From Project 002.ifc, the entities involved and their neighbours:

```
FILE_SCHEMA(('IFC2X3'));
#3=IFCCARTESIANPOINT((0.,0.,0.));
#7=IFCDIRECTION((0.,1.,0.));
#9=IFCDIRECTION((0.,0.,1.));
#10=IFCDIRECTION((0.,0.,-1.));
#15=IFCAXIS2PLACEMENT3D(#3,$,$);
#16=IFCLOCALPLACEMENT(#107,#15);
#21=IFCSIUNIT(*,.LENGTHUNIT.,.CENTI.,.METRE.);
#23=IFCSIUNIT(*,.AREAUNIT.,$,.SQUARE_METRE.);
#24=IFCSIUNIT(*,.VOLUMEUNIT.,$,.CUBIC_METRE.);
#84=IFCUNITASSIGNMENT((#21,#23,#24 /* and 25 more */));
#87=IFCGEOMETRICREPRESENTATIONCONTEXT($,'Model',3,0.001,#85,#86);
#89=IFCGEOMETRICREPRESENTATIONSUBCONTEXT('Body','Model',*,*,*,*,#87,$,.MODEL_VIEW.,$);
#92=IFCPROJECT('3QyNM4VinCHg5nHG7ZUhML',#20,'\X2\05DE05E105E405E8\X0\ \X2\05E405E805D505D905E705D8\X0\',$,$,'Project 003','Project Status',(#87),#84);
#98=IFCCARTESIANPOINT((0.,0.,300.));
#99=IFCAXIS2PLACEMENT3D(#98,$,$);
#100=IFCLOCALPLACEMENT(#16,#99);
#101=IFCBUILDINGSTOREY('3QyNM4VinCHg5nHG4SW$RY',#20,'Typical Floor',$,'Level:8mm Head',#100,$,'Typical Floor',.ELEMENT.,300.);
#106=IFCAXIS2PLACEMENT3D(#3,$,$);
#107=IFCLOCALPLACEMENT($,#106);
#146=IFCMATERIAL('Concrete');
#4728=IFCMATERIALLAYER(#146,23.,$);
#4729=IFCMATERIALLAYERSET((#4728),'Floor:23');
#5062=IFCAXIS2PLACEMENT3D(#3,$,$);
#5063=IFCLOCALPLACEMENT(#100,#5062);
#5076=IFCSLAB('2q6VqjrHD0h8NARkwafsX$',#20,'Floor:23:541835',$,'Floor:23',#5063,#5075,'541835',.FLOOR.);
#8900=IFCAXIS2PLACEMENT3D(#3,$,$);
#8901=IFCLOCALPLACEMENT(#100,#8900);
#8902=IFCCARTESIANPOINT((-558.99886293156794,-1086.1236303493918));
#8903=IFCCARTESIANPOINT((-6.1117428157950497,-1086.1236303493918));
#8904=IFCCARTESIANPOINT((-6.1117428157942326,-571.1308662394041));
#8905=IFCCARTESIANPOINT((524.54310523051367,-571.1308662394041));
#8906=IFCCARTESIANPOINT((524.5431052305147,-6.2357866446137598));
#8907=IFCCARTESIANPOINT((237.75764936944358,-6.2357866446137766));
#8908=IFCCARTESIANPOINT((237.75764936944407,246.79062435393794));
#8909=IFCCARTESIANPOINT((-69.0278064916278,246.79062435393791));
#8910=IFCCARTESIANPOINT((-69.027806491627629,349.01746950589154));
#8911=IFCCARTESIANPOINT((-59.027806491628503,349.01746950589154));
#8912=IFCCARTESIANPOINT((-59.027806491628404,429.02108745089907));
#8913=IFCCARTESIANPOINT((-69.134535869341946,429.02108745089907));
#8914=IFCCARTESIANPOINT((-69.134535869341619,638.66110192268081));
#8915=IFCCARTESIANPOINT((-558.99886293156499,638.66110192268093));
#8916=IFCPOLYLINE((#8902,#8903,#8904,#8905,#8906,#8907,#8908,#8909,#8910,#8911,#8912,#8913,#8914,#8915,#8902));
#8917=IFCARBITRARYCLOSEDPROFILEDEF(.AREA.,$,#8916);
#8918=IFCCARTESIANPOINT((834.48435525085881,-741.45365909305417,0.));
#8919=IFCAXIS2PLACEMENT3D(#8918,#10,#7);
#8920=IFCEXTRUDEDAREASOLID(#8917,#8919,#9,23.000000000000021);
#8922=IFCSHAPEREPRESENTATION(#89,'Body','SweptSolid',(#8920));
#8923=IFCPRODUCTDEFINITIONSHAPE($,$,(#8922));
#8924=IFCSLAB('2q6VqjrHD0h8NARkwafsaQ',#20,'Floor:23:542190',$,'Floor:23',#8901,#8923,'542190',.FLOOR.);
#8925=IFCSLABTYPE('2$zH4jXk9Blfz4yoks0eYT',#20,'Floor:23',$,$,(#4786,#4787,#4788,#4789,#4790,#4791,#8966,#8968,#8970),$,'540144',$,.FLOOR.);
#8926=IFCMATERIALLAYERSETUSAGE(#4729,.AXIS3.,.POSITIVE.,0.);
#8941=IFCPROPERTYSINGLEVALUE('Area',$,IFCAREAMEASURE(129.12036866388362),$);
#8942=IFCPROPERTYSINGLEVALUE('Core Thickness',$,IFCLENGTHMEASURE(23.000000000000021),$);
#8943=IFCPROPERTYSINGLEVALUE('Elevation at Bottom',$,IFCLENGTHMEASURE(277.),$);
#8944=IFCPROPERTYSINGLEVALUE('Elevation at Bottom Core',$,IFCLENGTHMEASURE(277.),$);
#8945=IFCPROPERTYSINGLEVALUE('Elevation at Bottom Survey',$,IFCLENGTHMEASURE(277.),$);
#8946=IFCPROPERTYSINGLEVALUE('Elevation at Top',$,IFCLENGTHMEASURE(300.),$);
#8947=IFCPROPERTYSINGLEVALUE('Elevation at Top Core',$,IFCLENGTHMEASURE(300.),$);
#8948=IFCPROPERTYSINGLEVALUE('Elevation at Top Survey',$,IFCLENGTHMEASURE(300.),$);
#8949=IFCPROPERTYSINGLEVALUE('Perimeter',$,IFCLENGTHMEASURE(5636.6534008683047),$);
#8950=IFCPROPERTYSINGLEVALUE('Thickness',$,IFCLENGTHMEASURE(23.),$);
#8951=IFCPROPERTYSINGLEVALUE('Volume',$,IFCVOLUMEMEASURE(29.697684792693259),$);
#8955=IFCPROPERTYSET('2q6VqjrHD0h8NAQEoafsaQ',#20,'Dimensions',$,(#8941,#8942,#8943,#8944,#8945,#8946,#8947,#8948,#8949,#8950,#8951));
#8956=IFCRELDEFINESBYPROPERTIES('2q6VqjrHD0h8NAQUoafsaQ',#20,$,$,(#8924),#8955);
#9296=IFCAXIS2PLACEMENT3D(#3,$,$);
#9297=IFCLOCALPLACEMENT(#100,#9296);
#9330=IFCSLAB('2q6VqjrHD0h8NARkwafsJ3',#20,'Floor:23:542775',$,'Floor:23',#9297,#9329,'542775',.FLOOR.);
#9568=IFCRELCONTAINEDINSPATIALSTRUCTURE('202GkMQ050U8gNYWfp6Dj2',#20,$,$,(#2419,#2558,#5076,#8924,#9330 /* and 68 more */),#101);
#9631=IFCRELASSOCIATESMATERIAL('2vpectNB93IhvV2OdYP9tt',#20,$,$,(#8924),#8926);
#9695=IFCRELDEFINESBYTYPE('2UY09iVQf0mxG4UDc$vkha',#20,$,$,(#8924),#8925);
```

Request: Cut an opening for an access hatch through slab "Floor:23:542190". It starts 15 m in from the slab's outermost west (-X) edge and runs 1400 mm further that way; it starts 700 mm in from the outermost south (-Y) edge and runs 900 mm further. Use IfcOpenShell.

```python
import numpy as np
import ifcopenshell
import ifcopenshell.api.feature
import ifcopenshell.api.geometry
import ifcopenshell.api.pset
import ifcopenshell.api.root
import ifcopenshell.geom
import ifcopenshell.util.element
import ifcopenshell.util.placement
import ifcopenshell.util.representation
import ifcopenshell.util.shape
import ifcopenshell.util.unit

model = ifcopenshell.open("Project 002.ifc")
unit_scale = ifcopenshell.util.unit.calculate_unit_scale(model)
area_scale = ifcopenshell.util.unit.calculate_unit_scale(model, "AREAUNIT")
volume_scale = ifcopenshell.util.unit.calculate_unit_scale(model, "VOLUMEUNIT")
settings = ifcopenshell.geom.settings()


def volume(element):
    """Net volume in cubic metres, openings subtracted."""
    shape = ifcopenshell.geom.create_shape(settings, element)
    return ifcopenshell.util.shape.get_volume(shape.geometry)


slab = model.by_id(8924)
before = volume(slab)

# Extent in the slab's own axes, in metres. The edges named are its -X and -Y sides.
slab_shape = ifcopenshell.geom.create_shape(settings, slab)
vertices = ifcopenshell.util.shape.get_vertices(slab_shape.geometry)
x_min, y_min, bottom = vertices.min(axis=0)
top = vertices[:, 2].max()

opening = ifcopenshell.api.root.create_entity(model, ifc_class="IfcOpeningElement", name="Access hatch opening")
context = ifcopenshell.util.representation.get_context(model, "Model", "Body", "MODEL_VIEW")
width, depth = 1.4, 0.9
outline = [(0.0, 0.0), (width, 0.0), (width, depth), (0.0, depth), (0.0, 0.0)]
# Overshoot both faces by 50 mm so the cut is clean.
shape = ifcopenshell.api.geometry.add_slab_representation(
    model, context=context, depth=top - bottom + 0.1, polyline=outline
)
ifcopenshell.api.geometry.assign_representation(model, product=opening, representation=shape)

matrix = ifcopenshell.util.placement.get_local_placement(slab.ObjectPlacement)
matrix[:, 3] = matrix @ np.append(np.array([x_min + 15, y_min + 0.7, bottom - 0.05]) / unit_scale, 1.0)
ifcopenshell.api.geometry.edit_object_placement(model, product=opening, matrix=matrix, is_si=False)
ifcopenshell.api.feature.add_feature(model, feature=opening, element=slab)

after = volume(slab)

# Update the slab's stored quantities.
pset = model.by_id(ifcopenshell.util.element.get_pset(slab, "Dimensions", should_inherit=False)["id"])
ifcopenshell.api.pset.edit_pset(model, pset=pset, properties={
    "Area": model.create_entity("IfcAreaMeasure", after / (top - bottom) / area_scale),
    "Volume": model.create_entity("IfcVolumeMeasure", after / volume_scale),
})

print(f"slab volume {before:.3f} -> {after:.3f} m3")

model.write("Project 002_v2.ifc")
```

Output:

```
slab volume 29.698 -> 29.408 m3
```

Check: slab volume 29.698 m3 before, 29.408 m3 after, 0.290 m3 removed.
